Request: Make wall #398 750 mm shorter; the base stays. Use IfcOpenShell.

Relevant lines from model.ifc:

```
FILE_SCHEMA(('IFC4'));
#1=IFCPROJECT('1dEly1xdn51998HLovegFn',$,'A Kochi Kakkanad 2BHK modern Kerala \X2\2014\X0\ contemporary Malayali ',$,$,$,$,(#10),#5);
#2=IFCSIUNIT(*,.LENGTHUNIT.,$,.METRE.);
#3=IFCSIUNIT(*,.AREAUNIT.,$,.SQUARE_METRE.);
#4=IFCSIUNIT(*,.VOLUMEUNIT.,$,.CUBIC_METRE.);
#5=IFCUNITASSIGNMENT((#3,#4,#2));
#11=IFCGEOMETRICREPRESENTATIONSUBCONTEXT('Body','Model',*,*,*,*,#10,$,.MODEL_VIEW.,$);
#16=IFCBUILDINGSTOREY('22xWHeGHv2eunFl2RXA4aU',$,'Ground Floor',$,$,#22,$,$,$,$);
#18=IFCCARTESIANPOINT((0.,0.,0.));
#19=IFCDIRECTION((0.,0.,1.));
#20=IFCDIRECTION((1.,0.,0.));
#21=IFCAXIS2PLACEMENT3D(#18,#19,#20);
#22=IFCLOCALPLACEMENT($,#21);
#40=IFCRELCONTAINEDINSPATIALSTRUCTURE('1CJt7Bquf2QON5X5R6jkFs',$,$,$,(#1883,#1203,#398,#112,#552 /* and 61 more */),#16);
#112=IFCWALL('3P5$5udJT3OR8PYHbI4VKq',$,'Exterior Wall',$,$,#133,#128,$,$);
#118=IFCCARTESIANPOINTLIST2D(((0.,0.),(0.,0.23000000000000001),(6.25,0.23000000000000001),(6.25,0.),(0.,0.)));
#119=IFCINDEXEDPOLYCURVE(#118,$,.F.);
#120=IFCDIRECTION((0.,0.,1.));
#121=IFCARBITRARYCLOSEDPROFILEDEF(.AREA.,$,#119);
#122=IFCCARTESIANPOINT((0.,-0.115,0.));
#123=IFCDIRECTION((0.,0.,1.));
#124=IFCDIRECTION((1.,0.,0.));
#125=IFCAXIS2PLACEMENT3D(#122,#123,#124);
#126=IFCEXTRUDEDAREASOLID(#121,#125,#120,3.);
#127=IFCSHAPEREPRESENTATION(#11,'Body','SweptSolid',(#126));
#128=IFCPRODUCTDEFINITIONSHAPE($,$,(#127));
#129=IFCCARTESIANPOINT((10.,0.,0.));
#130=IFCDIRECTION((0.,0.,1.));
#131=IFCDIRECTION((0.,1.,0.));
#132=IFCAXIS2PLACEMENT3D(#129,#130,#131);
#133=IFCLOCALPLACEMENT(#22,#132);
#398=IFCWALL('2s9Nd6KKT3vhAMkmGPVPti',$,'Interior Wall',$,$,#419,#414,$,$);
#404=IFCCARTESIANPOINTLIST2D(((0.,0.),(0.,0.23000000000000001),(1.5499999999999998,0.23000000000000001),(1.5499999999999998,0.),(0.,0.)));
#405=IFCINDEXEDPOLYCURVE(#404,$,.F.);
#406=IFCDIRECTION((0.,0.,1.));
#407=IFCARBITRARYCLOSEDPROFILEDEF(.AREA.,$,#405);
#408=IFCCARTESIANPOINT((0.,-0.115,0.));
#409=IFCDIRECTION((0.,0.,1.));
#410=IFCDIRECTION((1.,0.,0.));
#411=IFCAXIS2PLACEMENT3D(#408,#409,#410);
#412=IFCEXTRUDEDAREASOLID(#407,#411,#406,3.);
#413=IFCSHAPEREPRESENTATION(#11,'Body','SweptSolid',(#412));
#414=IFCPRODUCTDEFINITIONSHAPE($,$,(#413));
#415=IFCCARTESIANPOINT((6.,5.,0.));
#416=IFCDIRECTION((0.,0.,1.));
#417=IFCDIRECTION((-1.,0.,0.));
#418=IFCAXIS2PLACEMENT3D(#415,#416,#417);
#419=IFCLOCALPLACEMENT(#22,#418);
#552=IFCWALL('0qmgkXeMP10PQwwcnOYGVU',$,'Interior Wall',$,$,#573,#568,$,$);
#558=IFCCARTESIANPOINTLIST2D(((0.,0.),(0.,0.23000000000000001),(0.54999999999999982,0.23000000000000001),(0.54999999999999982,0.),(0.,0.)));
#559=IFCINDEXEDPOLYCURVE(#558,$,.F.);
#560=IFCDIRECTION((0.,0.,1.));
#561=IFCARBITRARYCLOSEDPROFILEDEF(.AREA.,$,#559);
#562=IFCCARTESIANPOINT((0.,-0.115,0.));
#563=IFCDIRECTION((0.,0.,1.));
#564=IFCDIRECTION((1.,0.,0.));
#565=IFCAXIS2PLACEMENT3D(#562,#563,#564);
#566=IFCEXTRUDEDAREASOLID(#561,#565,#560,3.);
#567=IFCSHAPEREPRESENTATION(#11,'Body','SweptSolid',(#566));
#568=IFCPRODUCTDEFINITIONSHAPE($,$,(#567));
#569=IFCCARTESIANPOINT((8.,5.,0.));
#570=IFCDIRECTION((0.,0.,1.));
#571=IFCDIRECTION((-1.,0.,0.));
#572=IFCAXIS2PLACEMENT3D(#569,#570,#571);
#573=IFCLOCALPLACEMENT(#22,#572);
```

```python
import ifcopenshell
import ifcopenshell.geom
import ifcopenshell.util.representation
import ifcopenshell.util.shape
import ifcopenshell.util.unit

model = ifcopenshell.open("model.ifc")
unit_scale = ifcopenshell.util.unit.calculate_unit_scale(model)
settings = ifcopenshell.geom.settings()


def volume(element):
    """Net volume in cubic metres, openings subtracted."""
    shape = ifcopenshell.geom.create_shape(settings, element)
    return ifcopenshell.util.shape.get_volume(shape.geometry)


wall = model.by_guid("2s9Nd6KKT3vhAMkmGPVPti")
before = volume(wall)

body = ifcopenshell.util.representation.get_representation(wall, "Model", "Body")
solid = body.Items[0]
old_height = solid.Depth
solid.Depth -= 0.75 / unit_scale
after = volume(wall)

print(f"height {old_height:g} -> {solid.Depth:g}, volume {before:.3f} -> {after:.3f} m3")

model.write("model_v2.ifc")
```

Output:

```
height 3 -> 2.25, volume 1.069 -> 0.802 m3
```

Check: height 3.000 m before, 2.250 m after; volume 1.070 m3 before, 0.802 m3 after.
